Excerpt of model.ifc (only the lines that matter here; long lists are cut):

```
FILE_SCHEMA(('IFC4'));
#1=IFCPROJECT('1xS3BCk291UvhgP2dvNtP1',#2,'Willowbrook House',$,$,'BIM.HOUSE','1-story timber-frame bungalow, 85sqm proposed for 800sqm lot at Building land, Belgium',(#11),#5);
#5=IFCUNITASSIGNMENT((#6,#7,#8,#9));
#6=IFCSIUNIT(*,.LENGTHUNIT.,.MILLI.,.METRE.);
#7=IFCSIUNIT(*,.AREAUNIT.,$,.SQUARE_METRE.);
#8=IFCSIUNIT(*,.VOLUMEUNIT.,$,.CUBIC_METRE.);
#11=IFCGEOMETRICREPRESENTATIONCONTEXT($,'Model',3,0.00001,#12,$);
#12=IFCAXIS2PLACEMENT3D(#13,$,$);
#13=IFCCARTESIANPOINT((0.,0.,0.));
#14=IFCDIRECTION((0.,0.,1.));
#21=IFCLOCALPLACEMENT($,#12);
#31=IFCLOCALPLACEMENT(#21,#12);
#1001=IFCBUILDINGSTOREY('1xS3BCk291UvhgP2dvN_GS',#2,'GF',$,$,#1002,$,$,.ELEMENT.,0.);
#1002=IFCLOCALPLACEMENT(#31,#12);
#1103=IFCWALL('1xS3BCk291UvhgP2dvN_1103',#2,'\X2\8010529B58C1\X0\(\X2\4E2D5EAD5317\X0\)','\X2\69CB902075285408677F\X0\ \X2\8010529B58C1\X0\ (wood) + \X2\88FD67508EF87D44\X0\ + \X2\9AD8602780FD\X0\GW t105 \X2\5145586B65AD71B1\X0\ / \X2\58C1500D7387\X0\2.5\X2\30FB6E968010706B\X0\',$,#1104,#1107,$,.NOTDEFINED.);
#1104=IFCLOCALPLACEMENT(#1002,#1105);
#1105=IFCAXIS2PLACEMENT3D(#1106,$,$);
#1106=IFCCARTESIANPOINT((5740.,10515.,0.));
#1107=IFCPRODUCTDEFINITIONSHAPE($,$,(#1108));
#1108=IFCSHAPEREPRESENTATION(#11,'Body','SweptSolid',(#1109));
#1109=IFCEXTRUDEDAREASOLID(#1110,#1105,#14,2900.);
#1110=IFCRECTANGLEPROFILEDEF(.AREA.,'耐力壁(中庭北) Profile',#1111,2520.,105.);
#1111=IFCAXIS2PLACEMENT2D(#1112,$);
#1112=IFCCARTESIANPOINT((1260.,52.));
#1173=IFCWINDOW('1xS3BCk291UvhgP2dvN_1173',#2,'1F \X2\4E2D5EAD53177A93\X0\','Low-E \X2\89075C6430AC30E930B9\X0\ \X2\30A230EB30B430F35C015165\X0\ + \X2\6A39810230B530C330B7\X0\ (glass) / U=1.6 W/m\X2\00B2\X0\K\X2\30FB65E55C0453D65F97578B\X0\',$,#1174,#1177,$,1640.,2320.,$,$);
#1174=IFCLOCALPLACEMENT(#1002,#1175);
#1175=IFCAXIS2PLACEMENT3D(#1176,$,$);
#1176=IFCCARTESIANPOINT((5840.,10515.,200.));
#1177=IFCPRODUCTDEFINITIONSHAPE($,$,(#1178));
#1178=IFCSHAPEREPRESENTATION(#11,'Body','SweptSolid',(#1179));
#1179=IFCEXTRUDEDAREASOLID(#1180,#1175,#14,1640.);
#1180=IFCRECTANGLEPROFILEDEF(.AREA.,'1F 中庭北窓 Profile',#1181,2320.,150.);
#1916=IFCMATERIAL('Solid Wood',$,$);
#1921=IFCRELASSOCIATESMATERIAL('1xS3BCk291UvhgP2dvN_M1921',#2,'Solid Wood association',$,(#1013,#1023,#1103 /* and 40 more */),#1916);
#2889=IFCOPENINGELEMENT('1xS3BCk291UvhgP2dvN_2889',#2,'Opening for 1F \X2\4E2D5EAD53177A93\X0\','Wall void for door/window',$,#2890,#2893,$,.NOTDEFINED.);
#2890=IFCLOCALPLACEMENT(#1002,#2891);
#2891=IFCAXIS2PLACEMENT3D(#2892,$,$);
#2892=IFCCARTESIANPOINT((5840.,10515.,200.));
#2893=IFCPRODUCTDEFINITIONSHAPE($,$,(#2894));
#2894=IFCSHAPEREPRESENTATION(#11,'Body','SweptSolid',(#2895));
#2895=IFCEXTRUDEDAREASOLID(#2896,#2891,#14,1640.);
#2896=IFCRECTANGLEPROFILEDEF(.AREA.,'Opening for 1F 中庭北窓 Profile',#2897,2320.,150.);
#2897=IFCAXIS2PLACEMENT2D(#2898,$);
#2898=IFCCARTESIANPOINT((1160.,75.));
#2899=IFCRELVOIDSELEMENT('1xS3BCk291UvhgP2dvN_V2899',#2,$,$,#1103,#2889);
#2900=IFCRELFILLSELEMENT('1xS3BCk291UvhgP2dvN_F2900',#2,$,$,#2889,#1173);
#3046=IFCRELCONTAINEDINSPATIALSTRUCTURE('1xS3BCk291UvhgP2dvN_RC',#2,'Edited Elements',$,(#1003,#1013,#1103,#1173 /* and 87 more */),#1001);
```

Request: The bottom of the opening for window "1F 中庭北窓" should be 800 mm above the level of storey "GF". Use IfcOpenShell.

```python
import numpy as np
import ifcopenshell
import ifcopenshell.api.geometry
import ifcopenshell.geom
import ifcopenshell.util.element
import ifcopenshell.util.placement
import ifcopenshell.util.shape
import ifcopenshell.util.unit

model = ifcopenshell.open("model.ifc")
unit_scale = ifcopenshell.util.unit.calculate_unit_scale(model)

window = model.by_guid("1xS3BCk291UvhgP2dvN_1173")
opening = window.FillsVoids[0].RelatingOpeningElement
storey = ifcopenshell.util.element.get_container(window, ifc_class="IfcBuildingStorey")
level = ifcopenshell.util.placement.get_local_placement(storey.ObjectPlacement)[2, 3]

# The opening's origin need not be at the sill, so measure its lowest point.
shape = ifcopenshell.geom.create_shape(ifcopenshell.geom.settings(), opening)
bottom = ifcopenshell.util.shape.get_shape_bottom_elevation(shape, shape.geometry) / unit_scale
dz = level + 800.0 - bottom

shift = np.array([0.0, 0.0, dz])
# The window is not placed relative to its opening, so move both.
for product in (opening, window):
    matrix = ifcopenshell.util.placement.get_local_placement(product.ObjectPlacement)
    matrix[:3, 3] += shift
    ifcopenshell.api.geometry.edit_object_placement(model, product=product, matrix=matrix, is_si=False)

print(f"moved by {dz * unit_scale:+.3f} m")

model.write("model_updated.ifc")
```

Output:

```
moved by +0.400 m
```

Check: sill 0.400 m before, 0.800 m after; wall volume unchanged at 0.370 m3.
